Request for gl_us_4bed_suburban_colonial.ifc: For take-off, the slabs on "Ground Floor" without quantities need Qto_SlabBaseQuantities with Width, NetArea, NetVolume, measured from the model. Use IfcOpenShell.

First a look at what the model holds.

```python
import ifcopenshell
import ifcopenshell.util.element
import ifcopenshell.util.unit

model = ifcopenshell.open("gl_us_4bed_suburban_colonial.ifc")
print(model.schema)
for unit_type in ("LENGTHUNIT", "AREAUNIT", "VOLUMEUNIT"):
    print(unit_type, ifcopenshell.util.unit.calculate_unit_scale(model, unit_type))
storey = next(s for s in model.by_type("IfcBuildingStorey") if s.Name == "Ground Floor")
slabs = [e for e in ifcopenshell.util.element.get_decomposition(storey) if e.is_a("IfcSlab")]
for e in sorted(slabs, key=lambda e: e.id()):
    print(e.id(), e.is_a(), e.Name, list(ifcopenshell.util.element.get_psets(e, qtos_only=True)), sep=" | ")
```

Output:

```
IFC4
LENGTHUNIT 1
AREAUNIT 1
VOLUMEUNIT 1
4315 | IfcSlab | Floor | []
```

```python
import ifcopenshell
import ifcopenshell.api.pset
import ifcopenshell.geom
import ifcopenshell.util.element
import ifcopenshell.util.shape
import ifcopenshell.util.unit

model = ifcopenshell.open("gl_us_4bed_suburban_colonial.ifc")
unit_scale = ifcopenshell.util.unit.calculate_unit_scale(model)
area_scale = ifcopenshell.util.unit.calculate_unit_scale(model, "AREAUNIT")
volume_scale = ifcopenshell.util.unit.calculate_unit_scale(model, "VOLUMEUNIT")
settings = ifcopenshell.geom.settings()

storey = next(s for s in model.by_type("IfcBuildingStorey") if s.Name == "Ground Floor")
slabs = [e for e in ifcopenshell.util.element.get_decomposition(storey) if e.is_a("IfcSlab")]

for e in sorted(slabs, key=lambda e: e.id()):
    if ifcopenshell.util.element.get_psets(e, qtos_only=True, should_inherit=False):
        continue
    # Geometry comes back in metres, in the element's own axes.
    shape = ifcopenshell.geom.create_shape(settings, e)
    values = {
        "Width": ifcopenshell.util.shape.get_z(shape.geometry) / unit_scale,
        "NetArea": ifcopenshell.util.shape.get_footprint_area(shape.geometry) / area_scale,
        "NetVolume": ifcopenshell.util.shape.get_volume(shape.geometry) / volume_scale,
    }
    qto = ifcopenshell.api.pset.add_qto(model, product=e, name="Qto_SlabBaseQuantities")
    ifcopenshell.api.pset.edit_qto(model, qto=qto, properties=values)
    print(e.id(), {k: round(v, 3) for k, v in values.items()})

model.write("gl_us_4bed_suburban_colonial_edited.ifc")
```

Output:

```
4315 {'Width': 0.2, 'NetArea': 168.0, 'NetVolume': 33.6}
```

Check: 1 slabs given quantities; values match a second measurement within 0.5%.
